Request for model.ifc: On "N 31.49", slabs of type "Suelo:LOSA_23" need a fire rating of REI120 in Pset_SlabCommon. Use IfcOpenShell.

First a look at what the model holds.

```python
import ifcopenshell
import ifcopenshell.util.element

model = ifcopenshell.open("model.ifc")
print(model.schema)
storey = next(s for s in model.by_type("IfcBuildingStorey") if s.Name == "N 31.49")
slabs = [e for e in ifcopenshell.util.element.get_decomposition(storey) if e.is_a("IfcSlab")]
seen = {}
for e in slabs:
    element_type = ifcopenshell.util.element.get_type(e)
    key = (element_type.Name if element_type != e and element_type else None, ifcopenshell.util.element.get_pset(e, "Pset_SlabCommon", "FireRating"))
    seen[key] = seen.get(key, 0) + 1
for (name, value), count in sorted(seen.items(), key=str):
    print(count, "x", name, "|", value)
```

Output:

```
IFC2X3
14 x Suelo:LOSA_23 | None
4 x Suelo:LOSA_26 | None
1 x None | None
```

```python
import ifcopenshell
import ifcopenshell.api.pset
import ifcopenshell.util.element

model = ifcopenshell.open("model.ifc")

storey = next(s for s in model.by_type("IfcBuildingStorey") if s.Name == "N 31.49")
slabs = [e for e in ifcopenshell.util.element.get_decomposition(storey) if e.is_a("IfcSlab")]

count = 0
for e in slabs:
    element_type = ifcopenshell.util.element.get_type(e)
    if element_type in (None, e) or element_type.Name != "Suelo:LOSA_23":
        continue
    # add_pset returns the element's existing set when there is one.
    pset = ifcopenshell.api.pset.add_pset(model, product=e, name="Pset_SlabCommon")
    ifcopenshell.api.pset.edit_pset(model, pset=pset, properties={"FireRating": "REI120"})
    count += 1

print(count, "slabs updated")

model.write("model_rev.ifc")
```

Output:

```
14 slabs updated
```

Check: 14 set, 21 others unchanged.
